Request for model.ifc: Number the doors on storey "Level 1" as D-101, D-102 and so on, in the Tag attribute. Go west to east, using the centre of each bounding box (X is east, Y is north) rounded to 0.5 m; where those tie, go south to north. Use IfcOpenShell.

First a look at what the model holds.

```python
import ifcopenshell
import ifcopenshell.util.element
import ifcopenshell.util.placement

model = ifcopenshell.open("model.ifc")
print(model.schema)
storey = next(s for s in model.by_type("IfcBuildingStorey") if s.Name == "Level 1")
doors = [e for e in ifcopenshell.util.element.get_decomposition(storey) if e.is_a("IfcDoor")]
for e in sorted(doors, key=lambda e: e.id()):
    origin = ifcopenshell.util.placement.get_local_placement(e.ObjectPlacement)[:3, 3]
    print(e.id(), e.Tag, e.Name, origin.round(2) + 0.0, sep=" | ")
```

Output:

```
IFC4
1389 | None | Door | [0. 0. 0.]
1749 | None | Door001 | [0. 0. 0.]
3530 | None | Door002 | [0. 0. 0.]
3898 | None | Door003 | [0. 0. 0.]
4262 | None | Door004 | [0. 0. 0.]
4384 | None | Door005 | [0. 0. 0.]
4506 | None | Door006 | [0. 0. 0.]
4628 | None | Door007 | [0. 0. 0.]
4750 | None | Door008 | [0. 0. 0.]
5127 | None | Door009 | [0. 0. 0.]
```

```python
import ifcopenshell
import ifcopenshell.geom
import ifcopenshell.util.element
import ifcopenshell.util.shape

model = ifcopenshell.open("model.ifc")
settings = ifcopenshell.geom.settings()
settings.set("use-world-coords", True)


def centre(element):
    shape = ifcopenshell.geom.create_shape(settings, element)
    return ifcopenshell.util.shape.get_bbox_centroid(shape.geometry)


storey = next(s for s in model.by_type("IfcBuildingStorey") if s.Name == "Level 1")
doors = [e for e in ifcopenshell.util.element.get_decomposition(storey) if e.is_a("IfcDoor")]

# Insertion points can sit at a corner or the storey origin, so sort by the geometry (in metres).
centres = {e: centre(e) for e in doors}
doors.sort(key=lambda e: (round(centres[e][0] / 0.5), centres[e][1]))

for i, e in enumerate(doors, start=1):
    number = f"D-1{i:02d}"
    e.Tag = number
    print(e.id(), number)

model.write("model_v2.ifc")
```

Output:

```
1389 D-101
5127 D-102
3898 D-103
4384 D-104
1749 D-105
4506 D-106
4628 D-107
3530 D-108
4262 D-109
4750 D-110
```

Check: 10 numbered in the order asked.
